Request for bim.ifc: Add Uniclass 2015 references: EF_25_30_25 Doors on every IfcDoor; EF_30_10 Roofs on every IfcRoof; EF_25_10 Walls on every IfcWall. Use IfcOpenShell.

First a look at what the model holds.

```python
import ifcopenshell

model = ifcopenshell.open("bim.ifc")
print(model.schema)
print("classifications:", [c.Name for c in model.by_type("IfcClassification")])
for ifc_class in ("IfcDoor", "IfcRoof", "IfcStair", "IfcWall", "IfcWindow"):
    print(ifc_class, len(model.by_type(ifc_class)))
```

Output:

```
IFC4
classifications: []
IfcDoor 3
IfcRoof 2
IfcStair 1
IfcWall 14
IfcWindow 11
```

```python
import ifcopenshell
import ifcopenshell.api.classification

model = ifcopenshell.open("bim.ifc")

system = ifcopenshell.api.classification.add_classification(model, classification="Uniclass 2015")

codes = {
    "IfcDoor": ("EF_25_30_25", "Doors"),
    "IfcRoof": ("EF_30_10", "Roofs"),
    "IfcWall": ("EF_25_10", "Walls"),
}
for ifc_class, (code, name) in codes.items():
    products = model.by_type(ifc_class)
    ifcopenshell.api.classification.add_reference(
        model, products=products, classification=system, identification=code, name=name
    )
    print(code, len(products))

model.write("bim_v2.ifc")
```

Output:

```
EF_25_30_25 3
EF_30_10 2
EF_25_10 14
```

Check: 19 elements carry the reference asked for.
